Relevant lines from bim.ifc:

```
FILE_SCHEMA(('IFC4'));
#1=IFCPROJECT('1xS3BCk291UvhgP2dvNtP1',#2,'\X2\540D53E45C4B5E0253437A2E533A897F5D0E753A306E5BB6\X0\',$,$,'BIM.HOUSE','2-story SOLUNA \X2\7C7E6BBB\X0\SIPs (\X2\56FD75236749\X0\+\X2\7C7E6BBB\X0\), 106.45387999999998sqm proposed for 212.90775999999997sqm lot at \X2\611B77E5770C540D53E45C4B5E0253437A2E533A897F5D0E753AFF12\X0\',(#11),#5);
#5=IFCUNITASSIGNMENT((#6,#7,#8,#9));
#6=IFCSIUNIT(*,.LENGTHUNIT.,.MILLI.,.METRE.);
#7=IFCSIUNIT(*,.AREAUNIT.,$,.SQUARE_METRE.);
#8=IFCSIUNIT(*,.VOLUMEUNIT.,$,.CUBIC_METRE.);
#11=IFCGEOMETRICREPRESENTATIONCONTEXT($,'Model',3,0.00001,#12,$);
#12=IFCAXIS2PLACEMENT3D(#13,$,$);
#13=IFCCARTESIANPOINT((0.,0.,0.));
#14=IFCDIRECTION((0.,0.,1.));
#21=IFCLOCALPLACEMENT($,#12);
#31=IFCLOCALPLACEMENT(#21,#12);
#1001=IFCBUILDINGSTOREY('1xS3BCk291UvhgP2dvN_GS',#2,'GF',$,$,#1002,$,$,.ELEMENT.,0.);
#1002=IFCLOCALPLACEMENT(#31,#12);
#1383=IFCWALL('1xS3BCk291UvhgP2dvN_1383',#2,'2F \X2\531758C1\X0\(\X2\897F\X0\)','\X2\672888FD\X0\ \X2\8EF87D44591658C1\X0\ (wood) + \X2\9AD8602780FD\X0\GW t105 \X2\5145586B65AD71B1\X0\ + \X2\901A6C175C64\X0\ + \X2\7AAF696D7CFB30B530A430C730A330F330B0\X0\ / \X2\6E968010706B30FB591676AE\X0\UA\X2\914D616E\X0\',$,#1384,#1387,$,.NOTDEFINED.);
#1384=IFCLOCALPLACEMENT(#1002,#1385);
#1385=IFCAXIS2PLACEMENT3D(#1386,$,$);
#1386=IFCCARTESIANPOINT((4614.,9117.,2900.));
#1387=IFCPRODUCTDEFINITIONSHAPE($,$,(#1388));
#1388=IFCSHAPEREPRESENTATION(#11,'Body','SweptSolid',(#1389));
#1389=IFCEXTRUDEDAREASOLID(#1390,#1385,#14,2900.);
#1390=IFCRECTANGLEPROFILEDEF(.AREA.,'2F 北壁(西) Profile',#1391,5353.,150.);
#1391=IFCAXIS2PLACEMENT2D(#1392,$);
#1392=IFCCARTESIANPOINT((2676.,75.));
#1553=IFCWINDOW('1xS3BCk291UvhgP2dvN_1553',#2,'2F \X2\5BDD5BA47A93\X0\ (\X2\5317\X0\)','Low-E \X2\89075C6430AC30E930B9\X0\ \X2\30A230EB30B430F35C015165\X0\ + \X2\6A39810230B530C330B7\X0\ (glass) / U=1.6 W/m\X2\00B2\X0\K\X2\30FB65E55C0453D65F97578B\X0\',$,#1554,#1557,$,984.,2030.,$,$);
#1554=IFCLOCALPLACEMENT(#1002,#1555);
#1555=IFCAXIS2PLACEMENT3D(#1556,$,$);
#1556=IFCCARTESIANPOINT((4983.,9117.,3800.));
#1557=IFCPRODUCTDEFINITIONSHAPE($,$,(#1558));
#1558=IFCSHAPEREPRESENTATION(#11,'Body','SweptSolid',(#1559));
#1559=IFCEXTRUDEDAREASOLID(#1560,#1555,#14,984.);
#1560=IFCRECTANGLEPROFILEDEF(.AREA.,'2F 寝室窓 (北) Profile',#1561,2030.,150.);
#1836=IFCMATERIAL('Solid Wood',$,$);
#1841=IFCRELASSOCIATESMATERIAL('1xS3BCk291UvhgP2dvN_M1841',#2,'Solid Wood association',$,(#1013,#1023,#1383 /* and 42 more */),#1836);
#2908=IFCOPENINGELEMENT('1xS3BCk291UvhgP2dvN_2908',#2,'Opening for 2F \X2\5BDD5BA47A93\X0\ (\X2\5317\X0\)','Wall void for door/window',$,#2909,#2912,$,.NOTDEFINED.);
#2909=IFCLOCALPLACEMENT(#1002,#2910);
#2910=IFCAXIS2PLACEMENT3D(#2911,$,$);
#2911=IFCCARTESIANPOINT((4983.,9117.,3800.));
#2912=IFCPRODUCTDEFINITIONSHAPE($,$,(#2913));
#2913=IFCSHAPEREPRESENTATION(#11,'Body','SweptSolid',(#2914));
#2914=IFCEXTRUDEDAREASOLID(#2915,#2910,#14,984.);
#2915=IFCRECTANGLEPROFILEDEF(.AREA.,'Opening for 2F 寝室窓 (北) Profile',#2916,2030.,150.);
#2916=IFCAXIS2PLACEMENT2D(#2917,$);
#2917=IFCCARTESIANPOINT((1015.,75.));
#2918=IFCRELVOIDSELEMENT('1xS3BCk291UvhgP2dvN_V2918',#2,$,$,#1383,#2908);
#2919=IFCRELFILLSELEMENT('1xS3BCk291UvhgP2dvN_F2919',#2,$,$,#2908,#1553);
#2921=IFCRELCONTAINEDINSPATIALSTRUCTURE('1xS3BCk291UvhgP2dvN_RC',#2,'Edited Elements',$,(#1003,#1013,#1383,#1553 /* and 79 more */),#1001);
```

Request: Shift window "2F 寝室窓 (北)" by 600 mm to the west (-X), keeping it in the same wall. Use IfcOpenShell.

```python
import ifcopenshell
import ifcopenshell.api.geometry
import ifcopenshell.util.placement

model = ifcopenshell.open("bim.ifc")

window = model.by_id(1553)
opening = window.FillsVoids[0].RelatingOpeningElement
wall = opening.VoidsElements[0].RelatingBuildingElement

wall_matrix = ifcopenshell.util.placement.get_local_placement(wall.ObjectPlacement)
shift = wall_matrix[:3, 0] * -600.0
before = ifcopenshell.util.placement.get_local_placement(window.ObjectPlacement)[:3, 3].copy()

# The window is not placed relative to its opening, so move both.
for product in (opening, window):
    matrix = ifcopenshell.util.placement.get_local_placement(product.ObjectPlacement)
    matrix[:3, 3] += shift
    ifcopenshell.api.geometry.edit_object_placement(model, product=product, matrix=matrix, is_si=False)

after = ifcopenshell.util.placement.get_local_placement(window.ObjectPlacement)[:3, 3]
print("window moved by", (after - before).round(3) + 0.0)

model.write("bim_v2.ifc")
```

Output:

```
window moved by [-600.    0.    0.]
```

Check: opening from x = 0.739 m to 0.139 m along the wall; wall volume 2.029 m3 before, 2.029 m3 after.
